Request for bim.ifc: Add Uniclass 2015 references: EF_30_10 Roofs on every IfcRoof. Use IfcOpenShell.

First a look at what the model holds.

```python
import ifcopenshell

model = ifcopenshell.open("bim.ifc")
print(model.schema)
print("classifications:", [c.Name for c in model.by_type("IfcClassification")])
for ifc_class in ("IfcDoor", "IfcRoof", "IfcStair", "IfcWall", "IfcWindow"):
    print(ifc_class, len(model.by_type(ifc_class)))
```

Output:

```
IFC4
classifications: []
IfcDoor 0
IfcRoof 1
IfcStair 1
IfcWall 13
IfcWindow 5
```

```python
import ifcopenshell
import ifcopenshell.api.classification

model = ifcopenshell.open("bim.ifc")

system = ifcopenshell.api.classification.add_classification(model, classification="Uniclass 2015")

codes = {
    "IfcRoof": ("EF_30_10", "Roofs"),
}
for ifc_class, (code, name) in codes.items():
    products = model.by_type(ifc_class)
    ifcopenshell.api.classification.add_reference(
        model, products=products, classification=system, identification=code, name=name
    )
    print(code, len(products))

model.write("bim-out.ifc")
```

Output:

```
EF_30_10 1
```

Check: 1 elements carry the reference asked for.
